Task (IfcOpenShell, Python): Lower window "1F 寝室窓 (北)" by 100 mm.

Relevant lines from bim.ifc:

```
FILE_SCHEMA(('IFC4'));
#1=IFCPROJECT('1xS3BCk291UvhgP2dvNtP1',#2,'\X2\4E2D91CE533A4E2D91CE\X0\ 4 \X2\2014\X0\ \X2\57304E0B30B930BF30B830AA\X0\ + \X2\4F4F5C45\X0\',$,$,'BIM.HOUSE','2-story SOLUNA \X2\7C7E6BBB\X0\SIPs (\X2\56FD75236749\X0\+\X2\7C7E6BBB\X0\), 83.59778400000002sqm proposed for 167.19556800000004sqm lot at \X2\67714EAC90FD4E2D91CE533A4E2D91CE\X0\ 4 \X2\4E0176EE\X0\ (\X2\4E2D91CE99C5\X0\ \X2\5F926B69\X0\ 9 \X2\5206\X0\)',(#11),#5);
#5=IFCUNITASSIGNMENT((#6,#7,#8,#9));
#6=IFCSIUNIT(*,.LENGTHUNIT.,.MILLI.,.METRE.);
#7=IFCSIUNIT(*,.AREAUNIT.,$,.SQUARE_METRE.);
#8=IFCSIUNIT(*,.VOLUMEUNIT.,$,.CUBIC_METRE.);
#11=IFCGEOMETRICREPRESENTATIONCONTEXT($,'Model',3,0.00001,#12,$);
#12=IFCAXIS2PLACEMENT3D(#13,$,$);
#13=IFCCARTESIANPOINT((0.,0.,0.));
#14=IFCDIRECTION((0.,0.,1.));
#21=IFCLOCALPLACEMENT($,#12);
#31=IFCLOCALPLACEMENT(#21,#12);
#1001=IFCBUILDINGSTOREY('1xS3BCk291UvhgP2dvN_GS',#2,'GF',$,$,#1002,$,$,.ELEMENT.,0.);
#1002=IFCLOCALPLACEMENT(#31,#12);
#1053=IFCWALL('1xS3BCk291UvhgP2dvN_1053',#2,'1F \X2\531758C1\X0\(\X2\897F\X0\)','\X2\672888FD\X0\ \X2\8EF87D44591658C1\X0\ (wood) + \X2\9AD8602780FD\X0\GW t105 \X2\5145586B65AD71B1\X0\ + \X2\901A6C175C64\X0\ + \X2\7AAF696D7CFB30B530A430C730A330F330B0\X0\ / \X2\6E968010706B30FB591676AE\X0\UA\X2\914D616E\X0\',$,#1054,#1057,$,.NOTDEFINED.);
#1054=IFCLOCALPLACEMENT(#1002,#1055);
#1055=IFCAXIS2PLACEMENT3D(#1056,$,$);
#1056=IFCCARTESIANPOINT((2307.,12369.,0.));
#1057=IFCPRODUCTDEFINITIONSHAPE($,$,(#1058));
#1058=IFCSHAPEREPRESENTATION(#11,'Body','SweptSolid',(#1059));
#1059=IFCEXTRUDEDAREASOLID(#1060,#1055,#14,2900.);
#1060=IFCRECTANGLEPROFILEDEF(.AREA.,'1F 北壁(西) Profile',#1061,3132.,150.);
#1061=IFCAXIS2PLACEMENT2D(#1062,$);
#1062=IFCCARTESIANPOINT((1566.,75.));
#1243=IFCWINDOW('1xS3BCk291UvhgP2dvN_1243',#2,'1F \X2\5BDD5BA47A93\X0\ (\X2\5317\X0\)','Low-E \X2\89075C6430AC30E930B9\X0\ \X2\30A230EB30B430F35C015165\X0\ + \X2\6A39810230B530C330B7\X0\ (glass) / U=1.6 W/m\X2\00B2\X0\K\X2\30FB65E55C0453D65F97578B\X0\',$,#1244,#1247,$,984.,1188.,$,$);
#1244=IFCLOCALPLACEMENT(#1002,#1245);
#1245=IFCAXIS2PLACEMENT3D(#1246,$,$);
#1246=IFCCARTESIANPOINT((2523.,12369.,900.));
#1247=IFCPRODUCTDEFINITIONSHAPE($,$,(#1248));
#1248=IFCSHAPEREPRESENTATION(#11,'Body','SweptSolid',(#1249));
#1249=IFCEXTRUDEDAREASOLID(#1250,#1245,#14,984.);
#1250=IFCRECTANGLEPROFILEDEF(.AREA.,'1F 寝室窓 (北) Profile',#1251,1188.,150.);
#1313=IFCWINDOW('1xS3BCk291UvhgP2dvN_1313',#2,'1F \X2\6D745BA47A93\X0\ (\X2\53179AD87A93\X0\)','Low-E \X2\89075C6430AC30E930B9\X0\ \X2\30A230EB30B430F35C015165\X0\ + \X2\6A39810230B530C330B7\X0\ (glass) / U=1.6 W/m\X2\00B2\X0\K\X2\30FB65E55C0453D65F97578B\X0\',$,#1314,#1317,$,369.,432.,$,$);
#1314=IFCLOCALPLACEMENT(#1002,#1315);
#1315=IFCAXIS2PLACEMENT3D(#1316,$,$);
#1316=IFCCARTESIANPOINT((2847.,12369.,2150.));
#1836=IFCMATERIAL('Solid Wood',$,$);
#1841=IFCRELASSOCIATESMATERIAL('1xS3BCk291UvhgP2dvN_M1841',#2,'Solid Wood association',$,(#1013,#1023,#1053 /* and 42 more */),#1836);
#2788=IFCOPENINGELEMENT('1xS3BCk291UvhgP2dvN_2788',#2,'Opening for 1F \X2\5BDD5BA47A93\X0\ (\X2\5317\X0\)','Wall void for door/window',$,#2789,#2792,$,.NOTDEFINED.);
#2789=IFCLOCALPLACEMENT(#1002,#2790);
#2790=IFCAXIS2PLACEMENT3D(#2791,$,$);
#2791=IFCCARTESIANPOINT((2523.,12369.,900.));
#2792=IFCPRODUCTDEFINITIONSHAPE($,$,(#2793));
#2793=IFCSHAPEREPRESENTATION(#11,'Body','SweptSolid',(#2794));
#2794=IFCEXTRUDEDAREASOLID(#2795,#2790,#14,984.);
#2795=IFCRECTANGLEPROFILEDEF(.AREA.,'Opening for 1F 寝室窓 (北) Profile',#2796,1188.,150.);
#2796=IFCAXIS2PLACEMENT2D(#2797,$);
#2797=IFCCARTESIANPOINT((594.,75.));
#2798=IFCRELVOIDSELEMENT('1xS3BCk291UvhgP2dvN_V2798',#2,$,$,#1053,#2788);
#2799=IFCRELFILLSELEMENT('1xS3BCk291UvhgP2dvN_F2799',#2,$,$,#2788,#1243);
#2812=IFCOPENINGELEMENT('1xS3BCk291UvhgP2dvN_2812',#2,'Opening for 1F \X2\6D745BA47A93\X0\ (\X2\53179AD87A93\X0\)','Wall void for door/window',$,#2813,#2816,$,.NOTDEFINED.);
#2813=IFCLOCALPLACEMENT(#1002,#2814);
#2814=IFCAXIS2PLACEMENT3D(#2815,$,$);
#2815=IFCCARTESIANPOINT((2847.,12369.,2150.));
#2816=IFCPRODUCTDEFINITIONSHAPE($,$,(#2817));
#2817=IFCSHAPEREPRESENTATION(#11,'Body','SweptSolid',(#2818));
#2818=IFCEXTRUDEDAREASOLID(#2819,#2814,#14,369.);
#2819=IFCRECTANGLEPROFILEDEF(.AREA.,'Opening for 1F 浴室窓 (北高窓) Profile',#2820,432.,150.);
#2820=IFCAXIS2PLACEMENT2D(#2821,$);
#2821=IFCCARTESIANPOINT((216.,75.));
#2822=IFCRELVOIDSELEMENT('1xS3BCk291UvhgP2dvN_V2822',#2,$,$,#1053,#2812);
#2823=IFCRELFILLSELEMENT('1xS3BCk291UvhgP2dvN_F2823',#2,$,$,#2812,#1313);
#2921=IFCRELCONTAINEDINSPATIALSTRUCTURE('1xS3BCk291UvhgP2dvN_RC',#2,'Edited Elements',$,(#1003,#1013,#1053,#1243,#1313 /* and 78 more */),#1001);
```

```python
import numpy as np
import ifcopenshell
import ifcopenshell.api.geometry
import ifcopenshell.util.placement
import ifcopenshell.util.unit

model = ifcopenshell.open("bim.ifc")
unit_scale = ifcopenshell.util.unit.calculate_unit_scale(model)

window = model.by_id(1243)
opening = window.FillsVoids[0].RelatingOpeningElement
dz = -0.1 / unit_scale

shift = np.array([0.0, 0.0, dz])
# The window is not placed relative to its opening, so move both.
for product in (opening, window):
    matrix = ifcopenshell.util.placement.get_local_placement(product.ObjectPlacement)
    matrix[:3, 3] += shift
    ifcopenshell.api.geometry.edit_object_placement(model, product=product, matrix=matrix, is_si=False)

print(f"moved by {dz * unit_scale:+.3f} m")

model.write("bim_edited.ifc")
```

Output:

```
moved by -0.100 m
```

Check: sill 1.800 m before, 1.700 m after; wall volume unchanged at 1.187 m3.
